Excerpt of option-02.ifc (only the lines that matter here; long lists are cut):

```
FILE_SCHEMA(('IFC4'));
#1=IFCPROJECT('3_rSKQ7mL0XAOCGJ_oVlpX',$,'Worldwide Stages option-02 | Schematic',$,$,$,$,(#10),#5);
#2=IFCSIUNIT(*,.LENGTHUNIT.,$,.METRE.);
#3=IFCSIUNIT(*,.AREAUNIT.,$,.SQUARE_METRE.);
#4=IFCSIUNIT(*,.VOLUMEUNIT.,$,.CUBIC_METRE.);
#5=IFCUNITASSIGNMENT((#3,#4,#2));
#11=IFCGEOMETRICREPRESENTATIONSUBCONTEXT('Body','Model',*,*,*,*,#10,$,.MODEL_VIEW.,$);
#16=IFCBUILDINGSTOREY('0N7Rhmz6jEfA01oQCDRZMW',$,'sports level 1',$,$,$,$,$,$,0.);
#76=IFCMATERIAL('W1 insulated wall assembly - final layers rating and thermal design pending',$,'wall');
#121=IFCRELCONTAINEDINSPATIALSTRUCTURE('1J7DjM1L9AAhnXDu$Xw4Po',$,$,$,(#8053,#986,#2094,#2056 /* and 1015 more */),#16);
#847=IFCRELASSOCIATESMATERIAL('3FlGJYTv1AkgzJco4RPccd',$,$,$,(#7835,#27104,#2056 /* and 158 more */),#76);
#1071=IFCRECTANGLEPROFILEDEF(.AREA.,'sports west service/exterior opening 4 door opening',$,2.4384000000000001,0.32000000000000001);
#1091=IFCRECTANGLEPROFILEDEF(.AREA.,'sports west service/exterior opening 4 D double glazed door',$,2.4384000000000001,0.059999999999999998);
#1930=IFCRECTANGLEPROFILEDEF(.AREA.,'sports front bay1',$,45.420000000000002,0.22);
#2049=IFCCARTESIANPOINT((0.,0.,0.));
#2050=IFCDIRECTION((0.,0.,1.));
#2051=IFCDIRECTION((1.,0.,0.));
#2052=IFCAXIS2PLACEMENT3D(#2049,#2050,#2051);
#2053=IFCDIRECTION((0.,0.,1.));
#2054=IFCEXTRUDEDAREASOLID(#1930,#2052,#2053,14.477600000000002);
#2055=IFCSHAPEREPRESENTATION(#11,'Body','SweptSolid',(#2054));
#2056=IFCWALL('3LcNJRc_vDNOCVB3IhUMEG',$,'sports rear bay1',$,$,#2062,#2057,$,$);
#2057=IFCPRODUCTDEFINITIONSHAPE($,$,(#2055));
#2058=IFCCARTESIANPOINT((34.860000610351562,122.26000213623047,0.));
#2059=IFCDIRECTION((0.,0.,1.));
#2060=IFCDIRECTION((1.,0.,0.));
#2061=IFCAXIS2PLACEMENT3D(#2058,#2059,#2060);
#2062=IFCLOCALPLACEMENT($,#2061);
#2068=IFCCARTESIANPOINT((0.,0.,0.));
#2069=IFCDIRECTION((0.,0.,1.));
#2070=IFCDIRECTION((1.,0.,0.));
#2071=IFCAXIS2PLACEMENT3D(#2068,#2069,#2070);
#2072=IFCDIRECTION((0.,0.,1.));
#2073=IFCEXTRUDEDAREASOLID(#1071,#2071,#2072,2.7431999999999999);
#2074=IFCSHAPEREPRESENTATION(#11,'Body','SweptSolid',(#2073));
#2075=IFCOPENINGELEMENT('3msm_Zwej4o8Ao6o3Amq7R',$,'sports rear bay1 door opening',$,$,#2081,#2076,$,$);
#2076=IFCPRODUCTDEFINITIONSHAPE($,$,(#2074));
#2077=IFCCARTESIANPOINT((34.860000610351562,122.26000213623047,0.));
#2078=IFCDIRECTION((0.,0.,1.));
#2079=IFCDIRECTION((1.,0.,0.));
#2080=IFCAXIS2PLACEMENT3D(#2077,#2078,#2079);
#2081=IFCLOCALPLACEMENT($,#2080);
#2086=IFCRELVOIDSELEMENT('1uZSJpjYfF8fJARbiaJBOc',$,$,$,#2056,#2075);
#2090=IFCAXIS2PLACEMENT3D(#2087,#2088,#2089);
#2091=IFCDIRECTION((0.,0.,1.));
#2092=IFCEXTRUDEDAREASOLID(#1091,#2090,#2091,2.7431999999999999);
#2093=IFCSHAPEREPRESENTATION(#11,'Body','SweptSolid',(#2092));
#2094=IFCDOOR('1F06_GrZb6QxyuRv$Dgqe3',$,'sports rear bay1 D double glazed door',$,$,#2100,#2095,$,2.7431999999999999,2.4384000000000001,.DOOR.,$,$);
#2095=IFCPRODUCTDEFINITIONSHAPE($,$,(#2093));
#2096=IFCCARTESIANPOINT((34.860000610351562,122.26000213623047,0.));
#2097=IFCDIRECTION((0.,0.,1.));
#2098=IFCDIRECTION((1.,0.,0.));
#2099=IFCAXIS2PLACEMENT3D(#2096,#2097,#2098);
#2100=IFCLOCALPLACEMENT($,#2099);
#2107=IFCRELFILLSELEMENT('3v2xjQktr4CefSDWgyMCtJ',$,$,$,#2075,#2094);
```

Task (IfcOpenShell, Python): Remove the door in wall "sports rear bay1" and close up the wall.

```python
import ifcopenshell
import ifcopenshell.api.feature
import ifcopenshell.api.root
import ifcopenshell.geom
import ifcopenshell.util.shape

model = ifcopenshell.open("option-02.ifc")
settings = ifcopenshell.geom.settings()


def volume(element):
    """Net volume in cubic metres, openings subtracted."""
    shape = ifcopenshell.geom.create_shape(settings, element)
    return ifcopenshell.util.shape.get_volume(shape.geometry)


door = model.by_guid("1F06_GrZb6QxyuRv$Dgqe3")
opening = door.FillsVoids[0].RelatingOpeningElement
wall = opening.VoidsElements[0].RelatingBuildingElement
before = volume(wall)

ifcopenshell.api.root.remove_product(model, product=door)
ifcopenshell.api.feature.remove_feature(model, feature=opening)

after = volume(wall)

print(f"wall volume {before:.3f} -> {after:.3f} m3")

model.write("option-02_edited.ifc")
```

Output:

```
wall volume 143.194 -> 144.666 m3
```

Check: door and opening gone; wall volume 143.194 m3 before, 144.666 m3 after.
